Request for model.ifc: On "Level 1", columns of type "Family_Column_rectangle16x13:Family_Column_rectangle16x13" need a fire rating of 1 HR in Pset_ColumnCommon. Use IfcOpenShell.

First a look at what the model holds.

```python
import ifcopenshell
import ifcopenshell.util.element

model = ifcopenshell.open("model.ifc")
print(model.schema)
storey = next(s for s in model.by_type("IfcBuildingStorey") if s.Name == "Level 1")
columns = [e for e in ifcopenshell.util.element.get_decomposition(storey) if e.is_a("IfcColumn")]
seen = {}
for e in columns:
    element_type = ifcopenshell.util.element.get_type(e)
    key = (element_type.Name if element_type != e and element_type else None, ifcopenshell.util.element.get_pset(e, "Pset_ColumnCommon", "FireRating"))
    seen[key] = seen.get(key, 0) + 1
for (name, value), count in sorted(seen.items(), key=str):
    print(count, "x", name, "|", value)
```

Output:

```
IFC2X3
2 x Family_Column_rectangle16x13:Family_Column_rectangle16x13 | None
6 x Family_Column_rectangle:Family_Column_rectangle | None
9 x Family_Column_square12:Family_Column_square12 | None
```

```python
import ifcopenshell
import ifcopenshell.api.pset
import ifcopenshell.util.element

model = ifcopenshell.open("model.ifc")

storey = next(s for s in model.by_type("IfcBuildingStorey") if s.Name == "Level 1")
columns = [e for e in ifcopenshell.util.element.get_decomposition(storey) if e.is_a("IfcColumn")]

count = 0
for e in columns:
    element_type = ifcopenshell.util.element.get_type(e)
    if element_type in (None, e) or element_type.Name != "Family_Column_rectangle16x13:Family_Column_rectangle16x13":
        continue
    # add_pset returns the element's existing set when there is one.
    pset = ifcopenshell.api.pset.add_pset(model, product=e, name="Pset_ColumnCommon")
    ifcopenshell.api.pset.edit_pset(model, pset=pset, properties={"FireRating": "1 HR"})
    count += 1

print(count, "columns updated")

model.write("model_edited.ifc")
```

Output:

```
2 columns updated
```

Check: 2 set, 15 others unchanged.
